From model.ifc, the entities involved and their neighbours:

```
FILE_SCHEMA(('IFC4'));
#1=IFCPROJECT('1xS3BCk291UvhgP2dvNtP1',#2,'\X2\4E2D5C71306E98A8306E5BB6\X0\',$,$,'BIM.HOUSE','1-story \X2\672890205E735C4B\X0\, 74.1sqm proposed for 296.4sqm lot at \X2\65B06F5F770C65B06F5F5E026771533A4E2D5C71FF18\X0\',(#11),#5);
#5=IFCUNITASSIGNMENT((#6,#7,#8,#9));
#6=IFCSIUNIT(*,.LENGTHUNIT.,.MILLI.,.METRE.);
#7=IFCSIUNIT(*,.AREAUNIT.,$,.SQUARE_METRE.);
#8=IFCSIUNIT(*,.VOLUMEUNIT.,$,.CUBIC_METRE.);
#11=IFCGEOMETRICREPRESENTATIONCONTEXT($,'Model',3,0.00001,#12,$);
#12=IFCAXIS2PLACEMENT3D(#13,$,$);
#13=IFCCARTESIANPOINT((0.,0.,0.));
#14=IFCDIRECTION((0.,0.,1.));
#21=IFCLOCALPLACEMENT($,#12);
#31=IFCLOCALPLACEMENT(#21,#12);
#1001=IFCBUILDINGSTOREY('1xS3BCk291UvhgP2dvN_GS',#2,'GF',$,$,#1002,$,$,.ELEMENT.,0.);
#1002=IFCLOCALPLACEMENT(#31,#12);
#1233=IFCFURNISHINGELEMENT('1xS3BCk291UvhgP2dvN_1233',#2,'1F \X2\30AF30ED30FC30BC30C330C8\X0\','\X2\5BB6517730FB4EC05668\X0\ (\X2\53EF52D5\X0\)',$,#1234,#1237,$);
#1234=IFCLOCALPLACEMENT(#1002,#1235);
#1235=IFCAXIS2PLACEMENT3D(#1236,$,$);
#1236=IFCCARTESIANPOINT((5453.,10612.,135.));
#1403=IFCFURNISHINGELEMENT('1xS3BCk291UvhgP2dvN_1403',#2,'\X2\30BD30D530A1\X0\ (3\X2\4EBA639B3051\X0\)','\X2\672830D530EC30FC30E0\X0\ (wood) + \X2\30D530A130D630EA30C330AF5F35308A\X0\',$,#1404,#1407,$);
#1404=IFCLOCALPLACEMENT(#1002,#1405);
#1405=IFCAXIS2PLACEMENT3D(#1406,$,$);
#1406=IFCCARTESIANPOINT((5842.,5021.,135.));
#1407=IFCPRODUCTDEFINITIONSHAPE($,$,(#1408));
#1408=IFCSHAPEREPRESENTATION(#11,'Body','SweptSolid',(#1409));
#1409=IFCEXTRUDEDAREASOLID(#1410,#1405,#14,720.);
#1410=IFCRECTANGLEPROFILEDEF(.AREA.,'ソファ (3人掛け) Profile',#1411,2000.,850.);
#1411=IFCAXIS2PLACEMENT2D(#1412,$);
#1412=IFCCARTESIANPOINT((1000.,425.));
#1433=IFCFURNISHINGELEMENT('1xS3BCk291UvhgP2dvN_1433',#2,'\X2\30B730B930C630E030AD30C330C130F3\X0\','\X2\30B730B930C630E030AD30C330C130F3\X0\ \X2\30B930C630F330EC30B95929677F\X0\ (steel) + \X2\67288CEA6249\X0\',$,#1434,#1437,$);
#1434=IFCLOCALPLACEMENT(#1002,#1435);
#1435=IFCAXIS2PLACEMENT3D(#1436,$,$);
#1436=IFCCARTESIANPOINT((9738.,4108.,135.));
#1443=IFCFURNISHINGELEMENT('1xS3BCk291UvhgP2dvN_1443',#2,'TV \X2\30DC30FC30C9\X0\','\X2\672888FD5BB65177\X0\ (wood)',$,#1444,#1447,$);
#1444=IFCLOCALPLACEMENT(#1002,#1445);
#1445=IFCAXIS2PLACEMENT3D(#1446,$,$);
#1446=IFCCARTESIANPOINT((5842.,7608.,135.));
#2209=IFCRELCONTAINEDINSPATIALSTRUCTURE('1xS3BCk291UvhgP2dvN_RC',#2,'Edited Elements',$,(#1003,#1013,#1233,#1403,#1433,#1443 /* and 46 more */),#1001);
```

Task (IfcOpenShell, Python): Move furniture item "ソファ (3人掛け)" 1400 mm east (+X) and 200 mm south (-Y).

```python
import ifcopenshell
import ifcopenshell.api.geometry
import ifcopenshell.util.placement
import ifcopenshell.util.unit

model = ifcopenshell.open("model.ifc")
unit_scale = ifcopenshell.util.unit.calculate_unit_scale(model)

item = model.by_id(1403)
matrix = ifcopenshell.util.placement.get_local_placement(item.ObjectPlacement)
matrix[0, 3] += 1.4 / unit_scale
matrix[1, 3] -= 0.2 / unit_scale
ifcopenshell.api.geometry.edit_object_placement(model, product=item, matrix=matrix, is_si=False)

print(ifcopenshell.util.placement.get_local_placement(item.ObjectPlacement).round(3) + 0.0)

model.write("model_v2.ifc")
```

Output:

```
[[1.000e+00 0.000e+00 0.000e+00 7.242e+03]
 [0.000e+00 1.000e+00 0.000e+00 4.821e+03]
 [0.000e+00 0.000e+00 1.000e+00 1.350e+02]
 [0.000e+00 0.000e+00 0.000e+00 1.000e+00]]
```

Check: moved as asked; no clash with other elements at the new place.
